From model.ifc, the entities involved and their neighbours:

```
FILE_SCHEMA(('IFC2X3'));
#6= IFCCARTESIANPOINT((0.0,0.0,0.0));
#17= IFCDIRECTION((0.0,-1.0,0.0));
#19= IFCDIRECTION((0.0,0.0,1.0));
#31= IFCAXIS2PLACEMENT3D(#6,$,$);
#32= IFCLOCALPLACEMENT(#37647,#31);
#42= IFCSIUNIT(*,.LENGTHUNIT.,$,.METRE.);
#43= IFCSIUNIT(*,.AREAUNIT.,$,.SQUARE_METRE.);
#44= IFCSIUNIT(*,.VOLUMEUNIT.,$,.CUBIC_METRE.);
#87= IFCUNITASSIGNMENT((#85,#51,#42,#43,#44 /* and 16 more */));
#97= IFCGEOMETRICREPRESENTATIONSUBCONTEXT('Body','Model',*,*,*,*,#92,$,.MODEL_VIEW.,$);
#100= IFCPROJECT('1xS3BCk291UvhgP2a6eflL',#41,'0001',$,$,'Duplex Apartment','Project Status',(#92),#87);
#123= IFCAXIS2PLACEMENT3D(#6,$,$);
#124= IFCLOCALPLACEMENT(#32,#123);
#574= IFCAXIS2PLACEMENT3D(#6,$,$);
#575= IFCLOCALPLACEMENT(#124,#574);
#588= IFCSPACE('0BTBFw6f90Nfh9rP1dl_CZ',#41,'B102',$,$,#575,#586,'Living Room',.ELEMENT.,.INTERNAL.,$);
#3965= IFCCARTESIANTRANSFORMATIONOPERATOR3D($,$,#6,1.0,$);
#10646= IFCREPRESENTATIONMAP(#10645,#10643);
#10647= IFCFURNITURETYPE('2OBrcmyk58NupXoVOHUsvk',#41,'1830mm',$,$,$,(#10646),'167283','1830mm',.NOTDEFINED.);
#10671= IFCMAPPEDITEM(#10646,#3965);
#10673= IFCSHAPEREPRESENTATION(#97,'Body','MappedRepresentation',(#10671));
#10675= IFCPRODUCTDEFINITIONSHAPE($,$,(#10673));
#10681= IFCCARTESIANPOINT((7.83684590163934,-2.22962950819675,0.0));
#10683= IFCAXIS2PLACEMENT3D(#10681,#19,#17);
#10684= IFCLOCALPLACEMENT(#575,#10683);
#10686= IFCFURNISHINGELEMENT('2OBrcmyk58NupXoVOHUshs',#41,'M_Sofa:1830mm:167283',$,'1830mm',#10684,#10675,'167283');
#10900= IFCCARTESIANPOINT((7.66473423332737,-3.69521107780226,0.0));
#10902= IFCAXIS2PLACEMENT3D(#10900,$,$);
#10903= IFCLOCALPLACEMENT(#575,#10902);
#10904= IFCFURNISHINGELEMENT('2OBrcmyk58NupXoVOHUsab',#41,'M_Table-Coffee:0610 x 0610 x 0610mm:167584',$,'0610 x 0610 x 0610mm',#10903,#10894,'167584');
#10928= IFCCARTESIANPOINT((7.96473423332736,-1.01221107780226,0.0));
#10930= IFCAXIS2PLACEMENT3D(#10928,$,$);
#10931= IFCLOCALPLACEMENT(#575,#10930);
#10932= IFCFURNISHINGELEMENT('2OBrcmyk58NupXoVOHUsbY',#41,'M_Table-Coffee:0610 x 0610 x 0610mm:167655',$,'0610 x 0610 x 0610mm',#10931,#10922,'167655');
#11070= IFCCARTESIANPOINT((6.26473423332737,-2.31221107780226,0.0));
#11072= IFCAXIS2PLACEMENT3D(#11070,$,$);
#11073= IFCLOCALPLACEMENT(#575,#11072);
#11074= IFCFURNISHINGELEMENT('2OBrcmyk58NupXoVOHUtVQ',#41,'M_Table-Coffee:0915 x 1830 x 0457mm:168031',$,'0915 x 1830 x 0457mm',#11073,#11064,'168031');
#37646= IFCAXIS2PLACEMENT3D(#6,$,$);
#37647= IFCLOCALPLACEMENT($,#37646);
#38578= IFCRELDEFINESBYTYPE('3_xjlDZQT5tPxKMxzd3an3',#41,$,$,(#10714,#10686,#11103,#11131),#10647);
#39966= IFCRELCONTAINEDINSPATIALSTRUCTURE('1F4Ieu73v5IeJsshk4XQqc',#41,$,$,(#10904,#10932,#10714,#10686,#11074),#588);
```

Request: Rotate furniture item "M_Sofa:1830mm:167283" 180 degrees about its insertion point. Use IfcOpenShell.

```python
import ifcopenshell
import ifcopenshell.api.geometry
import ifcopenshell.util.placement

model = ifcopenshell.open("model.ifc")

item = model.by_guid("2OBrcmyk58NupXoVOHUshs")
matrix = ifcopenshell.util.placement.get_local_placement(item.ObjectPlacement)
matrix = matrix @ ifcopenshell.util.placement.rotation(180, "Z")
ifcopenshell.api.geometry.edit_object_placement(model, product=item, matrix=matrix, is_si=False)

print(ifcopenshell.util.placement.get_local_placement(item.ObjectPlacement).round(3) + 0.0)

model.write("model_updated.ifc")
```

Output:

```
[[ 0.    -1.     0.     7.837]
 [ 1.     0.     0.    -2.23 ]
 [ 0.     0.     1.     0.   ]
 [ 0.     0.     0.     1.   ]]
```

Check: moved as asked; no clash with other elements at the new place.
